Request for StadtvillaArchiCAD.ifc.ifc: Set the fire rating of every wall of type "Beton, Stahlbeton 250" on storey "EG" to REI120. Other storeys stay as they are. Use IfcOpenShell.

First a look at what the model holds.

```python
import ifcopenshell
import ifcopenshell.util.element

model = ifcopenshell.open("StadtvillaArchiCAD.ifc.ifc")
print(model.schema)
storey = next(s for s in model.by_type("IfcBuildingStorey") if s.Name == "EG")
walls = [e for e in ifcopenshell.util.element.get_decomposition(storey) if e.is_a("IfcWall")]
seen = {}
for e in walls:
    element_type = ifcopenshell.util.element.get_type(e)
    key = (element_type.Name if element_type != e and element_type else None, ifcopenshell.util.element.get_pset(e, "Pset_WallCommon", "FireRating"))
    seen[key] = seen.get(key, 0) + 1
for (name, value), count in sorted(seen.items(), key=str):
    print(count, "x", name, "|", value)
```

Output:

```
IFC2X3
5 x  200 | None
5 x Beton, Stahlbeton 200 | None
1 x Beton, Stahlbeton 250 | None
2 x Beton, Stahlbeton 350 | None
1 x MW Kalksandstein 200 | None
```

```python
import ifcopenshell
import ifcopenshell.api.pset
import ifcopenshell.util.element

model = ifcopenshell.open("StadtvillaArchiCAD.ifc.ifc")

storey = next(s for s in model.by_type("IfcBuildingStorey") if s.Name == "EG")
walls = [e for e in ifcopenshell.util.element.get_decomposition(storey) if e.is_a("IfcWall")]

count = 0
for e in walls:
    element_type = ifcopenshell.util.element.get_type(e)
    if element_type in (None, e) or element_type.Name != "Beton, Stahlbeton 250":
        continue
    # add_pset returns the element's existing set when there is one.
    pset = ifcopenshell.api.pset.add_pset(model, product=e, name="Pset_WallCommon")
    ifcopenshell.api.pset.edit_pset(model, pset=pset, properties={"FireRating": "REI120"})
    count += 1

print(count, "walls updated")

model.write("StadtvillaArchiCAD.ifc_rev.ifc")
```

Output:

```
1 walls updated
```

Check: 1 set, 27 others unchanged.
